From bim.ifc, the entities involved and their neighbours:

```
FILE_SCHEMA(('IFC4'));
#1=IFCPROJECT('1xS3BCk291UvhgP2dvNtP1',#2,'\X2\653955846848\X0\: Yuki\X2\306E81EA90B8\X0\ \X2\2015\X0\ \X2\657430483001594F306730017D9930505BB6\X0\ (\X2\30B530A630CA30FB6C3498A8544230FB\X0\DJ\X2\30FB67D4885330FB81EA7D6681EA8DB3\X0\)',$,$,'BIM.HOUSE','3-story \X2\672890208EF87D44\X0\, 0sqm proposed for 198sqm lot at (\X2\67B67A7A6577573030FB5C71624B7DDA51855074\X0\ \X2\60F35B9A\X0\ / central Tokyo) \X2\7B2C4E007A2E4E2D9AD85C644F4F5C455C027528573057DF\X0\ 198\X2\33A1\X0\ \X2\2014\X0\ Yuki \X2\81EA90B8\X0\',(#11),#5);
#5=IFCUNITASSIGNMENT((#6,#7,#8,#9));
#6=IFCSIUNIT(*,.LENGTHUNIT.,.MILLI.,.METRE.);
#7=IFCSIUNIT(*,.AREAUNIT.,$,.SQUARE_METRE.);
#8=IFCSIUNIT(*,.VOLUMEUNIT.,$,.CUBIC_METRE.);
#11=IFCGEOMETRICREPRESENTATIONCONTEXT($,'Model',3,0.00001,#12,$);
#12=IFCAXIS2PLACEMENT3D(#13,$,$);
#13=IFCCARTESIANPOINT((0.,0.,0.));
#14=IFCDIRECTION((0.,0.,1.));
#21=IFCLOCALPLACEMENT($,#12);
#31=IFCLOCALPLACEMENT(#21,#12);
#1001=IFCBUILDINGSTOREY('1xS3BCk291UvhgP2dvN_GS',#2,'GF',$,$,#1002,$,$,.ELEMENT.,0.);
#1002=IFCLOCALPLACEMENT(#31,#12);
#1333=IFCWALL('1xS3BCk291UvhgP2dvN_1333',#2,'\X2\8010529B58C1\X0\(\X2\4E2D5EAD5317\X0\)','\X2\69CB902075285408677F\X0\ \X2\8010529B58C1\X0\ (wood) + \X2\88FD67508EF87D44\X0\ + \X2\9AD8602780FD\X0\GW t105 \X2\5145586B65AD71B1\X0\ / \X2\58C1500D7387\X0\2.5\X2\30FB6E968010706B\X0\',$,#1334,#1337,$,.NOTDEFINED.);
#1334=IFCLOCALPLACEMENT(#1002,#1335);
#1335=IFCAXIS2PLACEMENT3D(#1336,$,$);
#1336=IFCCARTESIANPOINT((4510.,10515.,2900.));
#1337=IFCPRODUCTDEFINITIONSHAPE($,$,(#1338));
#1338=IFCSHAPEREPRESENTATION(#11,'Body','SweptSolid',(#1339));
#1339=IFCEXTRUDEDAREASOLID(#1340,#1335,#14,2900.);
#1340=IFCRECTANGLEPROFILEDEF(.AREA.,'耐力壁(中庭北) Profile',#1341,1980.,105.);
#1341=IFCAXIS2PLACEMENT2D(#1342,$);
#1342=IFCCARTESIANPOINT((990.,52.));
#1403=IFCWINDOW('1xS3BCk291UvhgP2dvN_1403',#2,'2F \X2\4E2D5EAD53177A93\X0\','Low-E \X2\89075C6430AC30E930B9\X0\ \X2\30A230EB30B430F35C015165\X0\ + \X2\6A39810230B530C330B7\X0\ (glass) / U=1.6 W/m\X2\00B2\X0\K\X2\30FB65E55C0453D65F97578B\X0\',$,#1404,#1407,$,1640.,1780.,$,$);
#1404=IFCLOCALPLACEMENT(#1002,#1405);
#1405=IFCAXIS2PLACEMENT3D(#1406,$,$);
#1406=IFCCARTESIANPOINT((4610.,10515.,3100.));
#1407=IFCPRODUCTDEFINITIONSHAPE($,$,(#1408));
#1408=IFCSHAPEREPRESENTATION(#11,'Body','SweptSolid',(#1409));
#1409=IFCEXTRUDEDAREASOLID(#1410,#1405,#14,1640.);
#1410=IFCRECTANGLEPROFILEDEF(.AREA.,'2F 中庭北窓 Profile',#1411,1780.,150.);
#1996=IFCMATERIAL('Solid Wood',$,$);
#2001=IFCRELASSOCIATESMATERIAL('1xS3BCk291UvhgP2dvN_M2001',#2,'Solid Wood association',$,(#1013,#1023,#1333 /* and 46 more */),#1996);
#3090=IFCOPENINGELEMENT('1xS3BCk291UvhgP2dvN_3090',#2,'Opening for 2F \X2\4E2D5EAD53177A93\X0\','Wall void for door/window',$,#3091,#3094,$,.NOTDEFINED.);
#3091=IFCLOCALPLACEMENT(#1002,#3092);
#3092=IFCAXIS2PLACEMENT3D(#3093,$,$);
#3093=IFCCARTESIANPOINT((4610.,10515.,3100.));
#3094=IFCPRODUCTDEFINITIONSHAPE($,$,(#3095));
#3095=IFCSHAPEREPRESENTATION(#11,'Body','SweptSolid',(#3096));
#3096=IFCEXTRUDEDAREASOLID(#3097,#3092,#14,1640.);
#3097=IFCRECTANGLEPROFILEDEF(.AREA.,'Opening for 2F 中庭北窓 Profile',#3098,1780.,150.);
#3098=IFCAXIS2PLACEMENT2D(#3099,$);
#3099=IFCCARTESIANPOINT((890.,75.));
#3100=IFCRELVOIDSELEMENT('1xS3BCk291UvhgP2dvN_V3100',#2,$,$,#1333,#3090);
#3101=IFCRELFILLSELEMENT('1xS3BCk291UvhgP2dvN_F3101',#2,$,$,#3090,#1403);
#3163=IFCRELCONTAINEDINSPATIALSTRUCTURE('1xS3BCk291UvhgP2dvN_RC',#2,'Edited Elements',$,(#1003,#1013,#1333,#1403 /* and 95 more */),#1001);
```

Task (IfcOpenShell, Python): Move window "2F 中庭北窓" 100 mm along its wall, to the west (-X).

```python
import ifcopenshell
import ifcopenshell.api.geometry
import ifcopenshell.util.placement

model = ifcopenshell.open("bim.ifc")

window = model.by_guid("1xS3BCk291UvhgP2dvN_1403")
opening = window.FillsVoids[0].RelatingOpeningElement
wall = opening.VoidsElements[0].RelatingBuildingElement

wall_matrix = ifcopenshell.util.placement.get_local_placement(wall.ObjectPlacement)
shift = wall_matrix[:3, 0] * -100.0
before = ifcopenshell.util.placement.get_local_placement(window.ObjectPlacement)[:3, 3].copy()

# The window is not placed relative to its opening, so move both.
for product in (opening, window):
    matrix = ifcopenshell.util.placement.get_local_placement(product.ObjectPlacement)
    matrix[:3, 3] += shift
    ifcopenshell.api.geometry.edit_object_placement(model, product=product, matrix=matrix, is_si=False)

after = ifcopenshell.util.placement.get_local_placement(window.ObjectPlacement)[:3, 3]
print("window moved by", (after - before).round(3) + 0.0)

model.write("bim_v2.ifc")
```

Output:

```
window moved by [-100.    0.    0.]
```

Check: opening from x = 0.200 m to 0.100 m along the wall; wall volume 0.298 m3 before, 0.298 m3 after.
